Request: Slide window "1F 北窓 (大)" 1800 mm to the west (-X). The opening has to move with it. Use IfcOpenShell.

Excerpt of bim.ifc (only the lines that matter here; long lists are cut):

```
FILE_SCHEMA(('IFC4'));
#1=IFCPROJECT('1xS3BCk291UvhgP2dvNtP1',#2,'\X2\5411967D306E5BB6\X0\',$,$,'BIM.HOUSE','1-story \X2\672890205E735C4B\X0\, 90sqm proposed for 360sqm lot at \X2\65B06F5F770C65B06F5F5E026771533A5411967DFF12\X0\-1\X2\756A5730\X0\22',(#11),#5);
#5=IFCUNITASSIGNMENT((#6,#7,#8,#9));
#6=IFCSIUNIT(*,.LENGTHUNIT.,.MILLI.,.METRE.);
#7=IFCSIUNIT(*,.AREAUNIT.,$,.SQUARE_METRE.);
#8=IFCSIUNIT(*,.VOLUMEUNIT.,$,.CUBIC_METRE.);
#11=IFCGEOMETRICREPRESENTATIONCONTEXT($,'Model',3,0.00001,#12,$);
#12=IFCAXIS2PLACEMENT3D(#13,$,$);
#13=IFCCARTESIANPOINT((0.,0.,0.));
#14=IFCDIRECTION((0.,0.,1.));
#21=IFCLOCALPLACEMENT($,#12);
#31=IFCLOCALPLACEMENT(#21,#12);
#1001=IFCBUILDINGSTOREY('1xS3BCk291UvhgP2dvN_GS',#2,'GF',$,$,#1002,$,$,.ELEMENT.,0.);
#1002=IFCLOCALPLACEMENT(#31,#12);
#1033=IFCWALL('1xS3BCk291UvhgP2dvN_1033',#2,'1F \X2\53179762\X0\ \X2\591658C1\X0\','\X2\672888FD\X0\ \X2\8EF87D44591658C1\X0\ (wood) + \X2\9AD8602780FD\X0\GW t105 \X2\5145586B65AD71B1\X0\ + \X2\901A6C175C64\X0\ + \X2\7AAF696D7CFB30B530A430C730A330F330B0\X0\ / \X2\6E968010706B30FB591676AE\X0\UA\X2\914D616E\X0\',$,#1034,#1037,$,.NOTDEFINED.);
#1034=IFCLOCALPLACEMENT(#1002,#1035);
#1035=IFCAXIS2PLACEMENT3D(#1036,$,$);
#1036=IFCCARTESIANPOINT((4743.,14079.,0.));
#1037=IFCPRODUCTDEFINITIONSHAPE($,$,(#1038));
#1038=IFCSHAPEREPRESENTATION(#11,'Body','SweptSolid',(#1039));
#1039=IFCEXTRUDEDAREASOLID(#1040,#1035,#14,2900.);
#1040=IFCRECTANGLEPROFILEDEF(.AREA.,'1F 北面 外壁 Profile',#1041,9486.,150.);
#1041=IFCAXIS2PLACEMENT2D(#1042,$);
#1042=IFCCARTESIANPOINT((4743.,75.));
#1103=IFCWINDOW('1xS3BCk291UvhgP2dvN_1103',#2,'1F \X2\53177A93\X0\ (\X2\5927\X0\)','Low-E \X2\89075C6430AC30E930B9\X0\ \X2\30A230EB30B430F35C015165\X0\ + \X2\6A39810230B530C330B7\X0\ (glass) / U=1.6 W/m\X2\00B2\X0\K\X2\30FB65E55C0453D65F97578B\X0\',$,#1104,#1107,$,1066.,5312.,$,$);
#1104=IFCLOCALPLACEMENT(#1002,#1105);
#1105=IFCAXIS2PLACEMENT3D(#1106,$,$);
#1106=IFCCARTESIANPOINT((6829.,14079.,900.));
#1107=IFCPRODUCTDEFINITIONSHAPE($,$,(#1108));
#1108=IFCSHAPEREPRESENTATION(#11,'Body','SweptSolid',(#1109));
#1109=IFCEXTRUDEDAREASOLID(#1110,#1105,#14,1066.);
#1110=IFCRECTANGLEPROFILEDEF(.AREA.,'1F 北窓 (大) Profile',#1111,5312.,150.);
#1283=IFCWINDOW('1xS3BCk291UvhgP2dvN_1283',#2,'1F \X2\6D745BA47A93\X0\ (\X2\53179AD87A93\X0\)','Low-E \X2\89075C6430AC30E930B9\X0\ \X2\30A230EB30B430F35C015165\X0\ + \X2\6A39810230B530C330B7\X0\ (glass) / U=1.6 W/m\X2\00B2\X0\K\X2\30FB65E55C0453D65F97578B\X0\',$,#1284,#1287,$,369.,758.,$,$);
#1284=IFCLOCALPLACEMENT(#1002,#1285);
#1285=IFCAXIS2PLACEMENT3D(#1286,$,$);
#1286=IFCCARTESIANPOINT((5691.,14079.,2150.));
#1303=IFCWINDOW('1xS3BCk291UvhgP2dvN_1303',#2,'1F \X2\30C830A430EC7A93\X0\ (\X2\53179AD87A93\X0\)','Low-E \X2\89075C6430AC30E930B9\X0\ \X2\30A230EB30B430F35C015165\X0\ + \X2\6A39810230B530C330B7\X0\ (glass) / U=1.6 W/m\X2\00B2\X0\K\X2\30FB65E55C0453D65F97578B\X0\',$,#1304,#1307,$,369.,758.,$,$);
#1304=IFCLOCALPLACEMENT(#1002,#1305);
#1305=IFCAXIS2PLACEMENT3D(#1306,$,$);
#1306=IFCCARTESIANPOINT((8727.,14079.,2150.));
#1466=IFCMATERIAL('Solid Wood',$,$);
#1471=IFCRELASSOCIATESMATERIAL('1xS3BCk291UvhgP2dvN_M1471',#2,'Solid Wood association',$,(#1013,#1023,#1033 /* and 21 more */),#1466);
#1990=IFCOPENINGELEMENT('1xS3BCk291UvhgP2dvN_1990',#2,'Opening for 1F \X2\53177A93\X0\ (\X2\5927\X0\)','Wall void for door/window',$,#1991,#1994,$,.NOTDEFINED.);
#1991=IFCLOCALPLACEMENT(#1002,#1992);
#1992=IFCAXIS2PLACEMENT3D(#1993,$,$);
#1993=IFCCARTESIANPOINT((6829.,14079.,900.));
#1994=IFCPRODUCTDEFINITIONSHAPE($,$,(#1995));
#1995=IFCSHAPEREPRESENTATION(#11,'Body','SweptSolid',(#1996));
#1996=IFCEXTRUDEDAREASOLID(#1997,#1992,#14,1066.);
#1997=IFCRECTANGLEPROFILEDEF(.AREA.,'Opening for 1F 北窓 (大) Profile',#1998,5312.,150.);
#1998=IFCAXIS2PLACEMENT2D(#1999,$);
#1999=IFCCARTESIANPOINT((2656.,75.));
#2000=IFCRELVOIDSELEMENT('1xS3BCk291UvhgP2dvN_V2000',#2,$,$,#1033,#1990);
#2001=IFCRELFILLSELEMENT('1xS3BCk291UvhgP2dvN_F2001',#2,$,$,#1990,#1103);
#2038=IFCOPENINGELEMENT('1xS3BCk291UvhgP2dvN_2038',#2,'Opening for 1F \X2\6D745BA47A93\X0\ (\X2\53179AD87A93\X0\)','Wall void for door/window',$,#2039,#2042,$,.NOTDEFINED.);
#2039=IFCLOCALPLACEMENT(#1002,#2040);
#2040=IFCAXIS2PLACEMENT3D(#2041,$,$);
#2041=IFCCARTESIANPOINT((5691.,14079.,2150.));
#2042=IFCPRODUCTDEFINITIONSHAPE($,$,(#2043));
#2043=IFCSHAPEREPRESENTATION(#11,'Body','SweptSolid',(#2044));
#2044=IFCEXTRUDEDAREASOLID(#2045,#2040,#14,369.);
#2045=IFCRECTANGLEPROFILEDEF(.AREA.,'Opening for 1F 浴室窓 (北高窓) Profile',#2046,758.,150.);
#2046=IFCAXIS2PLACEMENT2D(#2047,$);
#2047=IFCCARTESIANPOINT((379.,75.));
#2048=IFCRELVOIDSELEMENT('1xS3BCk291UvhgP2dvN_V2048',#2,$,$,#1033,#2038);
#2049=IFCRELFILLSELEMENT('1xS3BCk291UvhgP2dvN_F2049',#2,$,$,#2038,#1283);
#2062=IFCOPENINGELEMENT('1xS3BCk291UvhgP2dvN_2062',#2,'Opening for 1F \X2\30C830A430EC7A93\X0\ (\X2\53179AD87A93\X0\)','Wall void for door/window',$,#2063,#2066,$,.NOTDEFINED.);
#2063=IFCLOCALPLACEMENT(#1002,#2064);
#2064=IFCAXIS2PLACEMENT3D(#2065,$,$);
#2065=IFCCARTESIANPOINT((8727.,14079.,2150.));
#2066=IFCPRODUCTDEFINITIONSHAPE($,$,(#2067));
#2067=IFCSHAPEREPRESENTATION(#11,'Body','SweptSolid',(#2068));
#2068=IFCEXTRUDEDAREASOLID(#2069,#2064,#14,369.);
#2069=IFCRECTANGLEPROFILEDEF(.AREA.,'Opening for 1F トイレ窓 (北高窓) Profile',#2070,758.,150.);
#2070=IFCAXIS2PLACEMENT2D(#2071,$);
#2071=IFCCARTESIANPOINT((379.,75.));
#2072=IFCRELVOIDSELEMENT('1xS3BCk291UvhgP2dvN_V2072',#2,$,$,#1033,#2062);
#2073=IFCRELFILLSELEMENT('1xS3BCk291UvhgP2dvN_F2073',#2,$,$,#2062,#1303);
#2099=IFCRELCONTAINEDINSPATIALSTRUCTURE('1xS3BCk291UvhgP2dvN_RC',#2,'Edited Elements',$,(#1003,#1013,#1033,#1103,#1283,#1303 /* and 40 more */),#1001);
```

```python
import ifcopenshell
import ifcopenshell.api.geometry
import ifcopenshell.util.placement
import ifcopenshell.util.unit

model = ifcopenshell.open("bim.ifc")
unit_scale = ifcopenshell.util.unit.calculate_unit_scale(model)

window = model.by_guid("1xS3BCk291UvhgP2dvN_1103")
opening = window.FillsVoids[0].RelatingOpeningElement
wall = opening.VoidsElements[0].RelatingBuildingElement

wall_matrix = ifcopenshell.util.placement.get_local_placement(wall.ObjectPlacement)
shift = wall_matrix[:3, 0] * -1.8 / unit_scale
before = ifcopenshell.util.placement.get_local_placement(window.ObjectPlacement)[:3, 3].copy()

# The window is not placed relative to its opening, so move both.
for product in (opening, window):
    matrix = ifcopenshell.util.placement.get_local_placement(product.ObjectPlacement)
    matrix[:3, 3] += shift
    ifcopenshell.api.geometry.edit_object_placement(model, product=product, matrix=matrix, is_si=False)

after = ifcopenshell.util.placement.get_local_placement(window.ObjectPlacement)[:3, 3]
print("window moved by", (after - before).round(3) + 0.0)

model.write("bim_rev.ifc")
```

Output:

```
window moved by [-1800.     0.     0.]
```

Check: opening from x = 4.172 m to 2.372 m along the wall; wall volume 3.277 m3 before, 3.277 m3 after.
